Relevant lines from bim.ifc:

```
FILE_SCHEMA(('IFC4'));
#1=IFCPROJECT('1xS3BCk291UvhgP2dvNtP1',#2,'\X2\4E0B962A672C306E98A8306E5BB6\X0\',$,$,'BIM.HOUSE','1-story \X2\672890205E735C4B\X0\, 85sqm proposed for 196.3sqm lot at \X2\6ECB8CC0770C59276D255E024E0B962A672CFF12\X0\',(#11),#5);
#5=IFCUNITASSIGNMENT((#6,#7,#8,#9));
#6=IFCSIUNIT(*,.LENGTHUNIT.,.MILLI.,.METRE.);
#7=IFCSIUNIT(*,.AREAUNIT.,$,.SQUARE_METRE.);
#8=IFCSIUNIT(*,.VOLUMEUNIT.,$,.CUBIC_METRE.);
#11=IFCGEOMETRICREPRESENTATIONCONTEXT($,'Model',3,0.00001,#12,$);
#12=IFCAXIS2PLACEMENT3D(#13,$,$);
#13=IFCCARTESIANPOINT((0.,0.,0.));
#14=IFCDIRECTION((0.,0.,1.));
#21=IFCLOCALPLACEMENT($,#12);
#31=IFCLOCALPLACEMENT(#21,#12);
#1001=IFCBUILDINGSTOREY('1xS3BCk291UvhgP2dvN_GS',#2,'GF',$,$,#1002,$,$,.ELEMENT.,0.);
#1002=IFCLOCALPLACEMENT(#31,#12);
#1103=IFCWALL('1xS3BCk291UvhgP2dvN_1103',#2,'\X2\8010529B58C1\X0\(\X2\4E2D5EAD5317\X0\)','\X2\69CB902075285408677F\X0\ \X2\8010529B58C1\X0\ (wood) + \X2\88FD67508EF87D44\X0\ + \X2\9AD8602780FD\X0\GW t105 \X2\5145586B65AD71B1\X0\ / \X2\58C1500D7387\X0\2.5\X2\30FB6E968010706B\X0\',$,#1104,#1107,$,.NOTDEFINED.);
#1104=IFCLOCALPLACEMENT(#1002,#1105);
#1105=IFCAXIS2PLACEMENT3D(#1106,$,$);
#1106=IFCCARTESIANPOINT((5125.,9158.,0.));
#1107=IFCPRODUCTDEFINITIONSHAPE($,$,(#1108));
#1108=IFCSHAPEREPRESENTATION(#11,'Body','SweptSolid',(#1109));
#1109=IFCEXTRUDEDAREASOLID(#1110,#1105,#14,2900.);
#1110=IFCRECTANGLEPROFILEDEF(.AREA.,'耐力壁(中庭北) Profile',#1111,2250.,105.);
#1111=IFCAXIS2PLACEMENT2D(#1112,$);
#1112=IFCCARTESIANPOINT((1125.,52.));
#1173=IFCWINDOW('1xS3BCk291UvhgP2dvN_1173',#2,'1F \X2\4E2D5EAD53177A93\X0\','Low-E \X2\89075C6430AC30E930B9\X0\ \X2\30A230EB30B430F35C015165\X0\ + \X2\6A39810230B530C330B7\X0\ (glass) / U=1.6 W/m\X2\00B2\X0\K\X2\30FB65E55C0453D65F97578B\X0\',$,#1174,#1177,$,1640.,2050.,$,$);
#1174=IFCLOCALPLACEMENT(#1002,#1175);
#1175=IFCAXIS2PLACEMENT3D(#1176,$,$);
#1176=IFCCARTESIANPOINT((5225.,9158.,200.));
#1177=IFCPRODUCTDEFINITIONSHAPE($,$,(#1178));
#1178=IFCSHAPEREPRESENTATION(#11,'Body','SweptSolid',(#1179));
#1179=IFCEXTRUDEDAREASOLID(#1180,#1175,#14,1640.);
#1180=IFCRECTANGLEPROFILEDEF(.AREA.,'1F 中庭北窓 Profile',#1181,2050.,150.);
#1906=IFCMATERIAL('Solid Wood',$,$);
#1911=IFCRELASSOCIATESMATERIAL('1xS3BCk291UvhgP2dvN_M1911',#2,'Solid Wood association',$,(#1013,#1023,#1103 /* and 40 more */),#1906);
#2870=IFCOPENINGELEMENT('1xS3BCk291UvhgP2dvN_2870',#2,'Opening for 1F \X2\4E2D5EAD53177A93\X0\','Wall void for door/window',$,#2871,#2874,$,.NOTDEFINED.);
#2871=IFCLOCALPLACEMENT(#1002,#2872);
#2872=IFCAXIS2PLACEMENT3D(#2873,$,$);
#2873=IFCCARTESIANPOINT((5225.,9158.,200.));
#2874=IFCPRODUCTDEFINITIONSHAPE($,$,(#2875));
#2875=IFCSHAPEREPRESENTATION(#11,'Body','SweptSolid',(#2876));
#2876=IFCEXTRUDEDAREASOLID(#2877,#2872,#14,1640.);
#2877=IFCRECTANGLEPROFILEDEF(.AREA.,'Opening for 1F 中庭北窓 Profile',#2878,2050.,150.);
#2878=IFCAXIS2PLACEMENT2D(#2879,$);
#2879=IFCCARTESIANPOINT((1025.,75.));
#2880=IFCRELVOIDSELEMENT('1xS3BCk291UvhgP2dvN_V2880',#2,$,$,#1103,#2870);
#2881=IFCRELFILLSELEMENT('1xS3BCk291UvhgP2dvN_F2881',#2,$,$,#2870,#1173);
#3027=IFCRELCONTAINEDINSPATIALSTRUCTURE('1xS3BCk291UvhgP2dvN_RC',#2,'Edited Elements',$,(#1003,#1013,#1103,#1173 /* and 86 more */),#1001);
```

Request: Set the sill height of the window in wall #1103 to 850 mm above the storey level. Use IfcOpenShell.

```python
import numpy as np
import ifcopenshell
import ifcopenshell.api.geometry
import ifcopenshell.geom
import ifcopenshell.util.element
import ifcopenshell.util.placement
import ifcopenshell.util.shape
import ifcopenshell.util.unit

model = ifcopenshell.open("bim.ifc")
unit_scale = ifcopenshell.util.unit.calculate_unit_scale(model)

window = model.by_guid("1xS3BCk291UvhgP2dvN_1173")
opening = window.FillsVoids[0].RelatingOpeningElement
storey = ifcopenshell.util.element.get_container(window, ifc_class="IfcBuildingStorey")
level = ifcopenshell.util.placement.get_local_placement(storey.ObjectPlacement)[2, 3]

# The opening's origin need not be at the sill, so measure its lowest point.
shape = ifcopenshell.geom.create_shape(ifcopenshell.geom.settings(), opening)
bottom = ifcopenshell.util.shape.get_shape_bottom_elevation(shape, shape.geometry) / unit_scale
dz = level + 850.0 - bottom

shift = np.array([0.0, 0.0, dz])
# The window is not placed relative to its opening, so move both.
for product in (opening, window):
    matrix = ifcopenshell.util.placement.get_local_placement(product.ObjectPlacement)
    matrix[:3, 3] += shift
    ifcopenshell.api.geometry.edit_object_placement(model, product=product, matrix=matrix, is_si=False)

print(f"moved by {dz * unit_scale:+.3f} m")

model.write("bim_v2.ifc")
```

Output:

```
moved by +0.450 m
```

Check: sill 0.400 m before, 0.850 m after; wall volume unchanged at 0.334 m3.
